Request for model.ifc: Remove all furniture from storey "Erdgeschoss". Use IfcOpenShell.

First a look at what the model holds.

```python
import ifcopenshell
import ifcopenshell.util.element

model = ifcopenshell.open("model.ifc")
print(model.schema)
storey = next(s for s in model.by_type("IfcBuildingStorey") if s.Name == "Erdgeschoss")
furniture = [e for e in ifcopenshell.util.element.get_decomposition(storey) if e.is_a("IfcFurnishingElement")]
seen = {}
for e in furniture:
    element_type = ifcopenshell.util.element.get_type(e)
    name = element_type.Name if element_type not in (None, e) else None
    seen[name] = seen.get(name, 0) + 1
for name, count in sorted(seen.items(), key=str):
    print(count, "x", name)
```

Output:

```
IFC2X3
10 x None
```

```python
import ifcopenshell
import ifcopenshell.api.root
import ifcopenshell.util.element

model = ifcopenshell.open("model.ifc")

storey = next(s for s in model.by_type("IfcBuildingStorey") if s.Name == "Erdgeschoss")
furniture = [e for e in ifcopenshell.util.element.get_decomposition(storey) if e.is_a("IfcFurnishingElement")]

for e in furniture:
    ifcopenshell.api.root.remove_product(model, product=e)
print(len(furniture), "removed")

model.write("model_updated.ifc")
```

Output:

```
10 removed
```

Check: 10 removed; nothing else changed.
